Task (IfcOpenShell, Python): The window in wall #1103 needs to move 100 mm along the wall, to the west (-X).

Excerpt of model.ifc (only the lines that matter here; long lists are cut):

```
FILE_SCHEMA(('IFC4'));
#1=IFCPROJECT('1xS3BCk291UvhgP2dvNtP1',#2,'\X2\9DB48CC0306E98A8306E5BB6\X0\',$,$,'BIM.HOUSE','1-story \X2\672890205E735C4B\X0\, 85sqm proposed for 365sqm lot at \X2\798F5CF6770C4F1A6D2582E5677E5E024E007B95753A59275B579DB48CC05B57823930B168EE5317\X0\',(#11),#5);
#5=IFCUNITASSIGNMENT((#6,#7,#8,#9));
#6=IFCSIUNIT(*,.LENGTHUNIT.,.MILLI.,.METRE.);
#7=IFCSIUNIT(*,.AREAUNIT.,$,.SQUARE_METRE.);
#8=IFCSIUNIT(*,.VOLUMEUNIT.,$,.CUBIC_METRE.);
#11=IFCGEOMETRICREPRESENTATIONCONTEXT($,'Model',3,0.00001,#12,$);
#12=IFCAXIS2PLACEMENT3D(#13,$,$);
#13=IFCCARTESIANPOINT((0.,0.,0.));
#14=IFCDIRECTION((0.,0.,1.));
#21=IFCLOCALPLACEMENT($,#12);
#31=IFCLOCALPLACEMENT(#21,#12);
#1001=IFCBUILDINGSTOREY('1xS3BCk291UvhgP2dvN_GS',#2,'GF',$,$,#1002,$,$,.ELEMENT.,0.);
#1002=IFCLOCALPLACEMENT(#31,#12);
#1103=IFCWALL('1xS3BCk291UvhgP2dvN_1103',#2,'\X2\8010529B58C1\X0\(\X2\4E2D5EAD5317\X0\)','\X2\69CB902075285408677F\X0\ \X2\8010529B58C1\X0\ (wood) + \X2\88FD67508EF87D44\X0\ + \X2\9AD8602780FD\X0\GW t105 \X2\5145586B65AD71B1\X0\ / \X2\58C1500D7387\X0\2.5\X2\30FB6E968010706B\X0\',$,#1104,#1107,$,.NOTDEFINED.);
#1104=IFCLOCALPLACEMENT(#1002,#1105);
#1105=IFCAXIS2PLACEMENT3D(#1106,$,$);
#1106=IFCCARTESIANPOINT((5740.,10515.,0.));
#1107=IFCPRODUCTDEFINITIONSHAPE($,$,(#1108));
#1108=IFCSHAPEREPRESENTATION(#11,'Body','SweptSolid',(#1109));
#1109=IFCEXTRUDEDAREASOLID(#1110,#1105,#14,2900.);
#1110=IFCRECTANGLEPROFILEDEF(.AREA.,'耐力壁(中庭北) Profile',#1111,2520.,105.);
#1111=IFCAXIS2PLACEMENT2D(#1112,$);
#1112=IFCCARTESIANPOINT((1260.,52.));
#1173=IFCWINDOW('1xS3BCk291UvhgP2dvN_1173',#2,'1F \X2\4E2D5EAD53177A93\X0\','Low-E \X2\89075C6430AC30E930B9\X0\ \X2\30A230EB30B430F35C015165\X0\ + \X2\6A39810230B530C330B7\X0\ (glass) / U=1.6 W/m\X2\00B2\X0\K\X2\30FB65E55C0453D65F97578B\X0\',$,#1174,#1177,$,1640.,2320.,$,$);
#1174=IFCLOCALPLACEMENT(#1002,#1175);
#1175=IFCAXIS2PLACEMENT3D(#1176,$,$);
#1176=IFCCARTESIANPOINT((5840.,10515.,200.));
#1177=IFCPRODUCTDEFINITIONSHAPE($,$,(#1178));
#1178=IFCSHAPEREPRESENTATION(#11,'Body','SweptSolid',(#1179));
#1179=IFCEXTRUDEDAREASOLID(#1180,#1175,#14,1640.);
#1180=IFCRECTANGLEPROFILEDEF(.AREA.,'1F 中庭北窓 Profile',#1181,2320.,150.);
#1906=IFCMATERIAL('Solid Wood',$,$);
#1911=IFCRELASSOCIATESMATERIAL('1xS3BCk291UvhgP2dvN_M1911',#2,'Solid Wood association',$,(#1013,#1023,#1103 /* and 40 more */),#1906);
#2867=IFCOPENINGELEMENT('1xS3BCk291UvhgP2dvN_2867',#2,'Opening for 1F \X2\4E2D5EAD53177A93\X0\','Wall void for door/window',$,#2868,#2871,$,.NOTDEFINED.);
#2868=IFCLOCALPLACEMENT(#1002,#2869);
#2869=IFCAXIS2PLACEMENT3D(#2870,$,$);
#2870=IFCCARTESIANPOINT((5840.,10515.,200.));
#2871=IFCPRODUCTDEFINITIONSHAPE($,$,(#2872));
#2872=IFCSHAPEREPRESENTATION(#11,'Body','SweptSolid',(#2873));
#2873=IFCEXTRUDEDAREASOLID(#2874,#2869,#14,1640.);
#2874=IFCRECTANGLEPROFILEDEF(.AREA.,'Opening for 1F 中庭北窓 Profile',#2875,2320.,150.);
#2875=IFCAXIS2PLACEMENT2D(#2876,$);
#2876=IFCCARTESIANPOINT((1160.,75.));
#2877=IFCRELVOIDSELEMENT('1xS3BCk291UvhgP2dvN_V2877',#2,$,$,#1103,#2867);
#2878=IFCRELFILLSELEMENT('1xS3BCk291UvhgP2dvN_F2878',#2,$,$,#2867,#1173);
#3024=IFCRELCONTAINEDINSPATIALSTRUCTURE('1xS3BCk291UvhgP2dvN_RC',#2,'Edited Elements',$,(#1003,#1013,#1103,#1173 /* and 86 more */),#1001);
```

```python
import ifcopenshell
import ifcopenshell.api.geometry
import ifcopenshell.util.placement
import ifcopenshell.util.unit

model = ifcopenshell.open("model.ifc")
unit_scale = ifcopenshell.util.unit.calculate_unit_scale(model)

window = model.by_id(1173)
opening = window.FillsVoids[0].RelatingOpeningElement
wall = opening.VoidsElements[0].RelatingBuildingElement

wall_matrix = ifcopenshell.util.placement.get_local_placement(wall.ObjectPlacement)
shift = wall_matrix[:3, 0] * -0.1 / unit_scale
before = ifcopenshell.util.placement.get_local_placement(window.ObjectPlacement)[:3, 3].copy()

# The window is not placed relative to its opening, so move both.
for product in (opening, window):
    matrix = ifcopenshell.util.placement.get_local_placement(product.ObjectPlacement)
    matrix[:3, 3] += shift
    ifcopenshell.api.geometry.edit_object_placement(model, product=product, matrix=matrix, is_si=False)

after = ifcopenshell.util.placement.get_local_placement(window.ObjectPlacement)[:3, 3]
print("window moved by", (after - before).round(3) + 0.0)

model.write("model_rev.ifc")
```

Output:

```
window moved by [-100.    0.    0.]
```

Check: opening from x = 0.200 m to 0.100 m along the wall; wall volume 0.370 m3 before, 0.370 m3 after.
